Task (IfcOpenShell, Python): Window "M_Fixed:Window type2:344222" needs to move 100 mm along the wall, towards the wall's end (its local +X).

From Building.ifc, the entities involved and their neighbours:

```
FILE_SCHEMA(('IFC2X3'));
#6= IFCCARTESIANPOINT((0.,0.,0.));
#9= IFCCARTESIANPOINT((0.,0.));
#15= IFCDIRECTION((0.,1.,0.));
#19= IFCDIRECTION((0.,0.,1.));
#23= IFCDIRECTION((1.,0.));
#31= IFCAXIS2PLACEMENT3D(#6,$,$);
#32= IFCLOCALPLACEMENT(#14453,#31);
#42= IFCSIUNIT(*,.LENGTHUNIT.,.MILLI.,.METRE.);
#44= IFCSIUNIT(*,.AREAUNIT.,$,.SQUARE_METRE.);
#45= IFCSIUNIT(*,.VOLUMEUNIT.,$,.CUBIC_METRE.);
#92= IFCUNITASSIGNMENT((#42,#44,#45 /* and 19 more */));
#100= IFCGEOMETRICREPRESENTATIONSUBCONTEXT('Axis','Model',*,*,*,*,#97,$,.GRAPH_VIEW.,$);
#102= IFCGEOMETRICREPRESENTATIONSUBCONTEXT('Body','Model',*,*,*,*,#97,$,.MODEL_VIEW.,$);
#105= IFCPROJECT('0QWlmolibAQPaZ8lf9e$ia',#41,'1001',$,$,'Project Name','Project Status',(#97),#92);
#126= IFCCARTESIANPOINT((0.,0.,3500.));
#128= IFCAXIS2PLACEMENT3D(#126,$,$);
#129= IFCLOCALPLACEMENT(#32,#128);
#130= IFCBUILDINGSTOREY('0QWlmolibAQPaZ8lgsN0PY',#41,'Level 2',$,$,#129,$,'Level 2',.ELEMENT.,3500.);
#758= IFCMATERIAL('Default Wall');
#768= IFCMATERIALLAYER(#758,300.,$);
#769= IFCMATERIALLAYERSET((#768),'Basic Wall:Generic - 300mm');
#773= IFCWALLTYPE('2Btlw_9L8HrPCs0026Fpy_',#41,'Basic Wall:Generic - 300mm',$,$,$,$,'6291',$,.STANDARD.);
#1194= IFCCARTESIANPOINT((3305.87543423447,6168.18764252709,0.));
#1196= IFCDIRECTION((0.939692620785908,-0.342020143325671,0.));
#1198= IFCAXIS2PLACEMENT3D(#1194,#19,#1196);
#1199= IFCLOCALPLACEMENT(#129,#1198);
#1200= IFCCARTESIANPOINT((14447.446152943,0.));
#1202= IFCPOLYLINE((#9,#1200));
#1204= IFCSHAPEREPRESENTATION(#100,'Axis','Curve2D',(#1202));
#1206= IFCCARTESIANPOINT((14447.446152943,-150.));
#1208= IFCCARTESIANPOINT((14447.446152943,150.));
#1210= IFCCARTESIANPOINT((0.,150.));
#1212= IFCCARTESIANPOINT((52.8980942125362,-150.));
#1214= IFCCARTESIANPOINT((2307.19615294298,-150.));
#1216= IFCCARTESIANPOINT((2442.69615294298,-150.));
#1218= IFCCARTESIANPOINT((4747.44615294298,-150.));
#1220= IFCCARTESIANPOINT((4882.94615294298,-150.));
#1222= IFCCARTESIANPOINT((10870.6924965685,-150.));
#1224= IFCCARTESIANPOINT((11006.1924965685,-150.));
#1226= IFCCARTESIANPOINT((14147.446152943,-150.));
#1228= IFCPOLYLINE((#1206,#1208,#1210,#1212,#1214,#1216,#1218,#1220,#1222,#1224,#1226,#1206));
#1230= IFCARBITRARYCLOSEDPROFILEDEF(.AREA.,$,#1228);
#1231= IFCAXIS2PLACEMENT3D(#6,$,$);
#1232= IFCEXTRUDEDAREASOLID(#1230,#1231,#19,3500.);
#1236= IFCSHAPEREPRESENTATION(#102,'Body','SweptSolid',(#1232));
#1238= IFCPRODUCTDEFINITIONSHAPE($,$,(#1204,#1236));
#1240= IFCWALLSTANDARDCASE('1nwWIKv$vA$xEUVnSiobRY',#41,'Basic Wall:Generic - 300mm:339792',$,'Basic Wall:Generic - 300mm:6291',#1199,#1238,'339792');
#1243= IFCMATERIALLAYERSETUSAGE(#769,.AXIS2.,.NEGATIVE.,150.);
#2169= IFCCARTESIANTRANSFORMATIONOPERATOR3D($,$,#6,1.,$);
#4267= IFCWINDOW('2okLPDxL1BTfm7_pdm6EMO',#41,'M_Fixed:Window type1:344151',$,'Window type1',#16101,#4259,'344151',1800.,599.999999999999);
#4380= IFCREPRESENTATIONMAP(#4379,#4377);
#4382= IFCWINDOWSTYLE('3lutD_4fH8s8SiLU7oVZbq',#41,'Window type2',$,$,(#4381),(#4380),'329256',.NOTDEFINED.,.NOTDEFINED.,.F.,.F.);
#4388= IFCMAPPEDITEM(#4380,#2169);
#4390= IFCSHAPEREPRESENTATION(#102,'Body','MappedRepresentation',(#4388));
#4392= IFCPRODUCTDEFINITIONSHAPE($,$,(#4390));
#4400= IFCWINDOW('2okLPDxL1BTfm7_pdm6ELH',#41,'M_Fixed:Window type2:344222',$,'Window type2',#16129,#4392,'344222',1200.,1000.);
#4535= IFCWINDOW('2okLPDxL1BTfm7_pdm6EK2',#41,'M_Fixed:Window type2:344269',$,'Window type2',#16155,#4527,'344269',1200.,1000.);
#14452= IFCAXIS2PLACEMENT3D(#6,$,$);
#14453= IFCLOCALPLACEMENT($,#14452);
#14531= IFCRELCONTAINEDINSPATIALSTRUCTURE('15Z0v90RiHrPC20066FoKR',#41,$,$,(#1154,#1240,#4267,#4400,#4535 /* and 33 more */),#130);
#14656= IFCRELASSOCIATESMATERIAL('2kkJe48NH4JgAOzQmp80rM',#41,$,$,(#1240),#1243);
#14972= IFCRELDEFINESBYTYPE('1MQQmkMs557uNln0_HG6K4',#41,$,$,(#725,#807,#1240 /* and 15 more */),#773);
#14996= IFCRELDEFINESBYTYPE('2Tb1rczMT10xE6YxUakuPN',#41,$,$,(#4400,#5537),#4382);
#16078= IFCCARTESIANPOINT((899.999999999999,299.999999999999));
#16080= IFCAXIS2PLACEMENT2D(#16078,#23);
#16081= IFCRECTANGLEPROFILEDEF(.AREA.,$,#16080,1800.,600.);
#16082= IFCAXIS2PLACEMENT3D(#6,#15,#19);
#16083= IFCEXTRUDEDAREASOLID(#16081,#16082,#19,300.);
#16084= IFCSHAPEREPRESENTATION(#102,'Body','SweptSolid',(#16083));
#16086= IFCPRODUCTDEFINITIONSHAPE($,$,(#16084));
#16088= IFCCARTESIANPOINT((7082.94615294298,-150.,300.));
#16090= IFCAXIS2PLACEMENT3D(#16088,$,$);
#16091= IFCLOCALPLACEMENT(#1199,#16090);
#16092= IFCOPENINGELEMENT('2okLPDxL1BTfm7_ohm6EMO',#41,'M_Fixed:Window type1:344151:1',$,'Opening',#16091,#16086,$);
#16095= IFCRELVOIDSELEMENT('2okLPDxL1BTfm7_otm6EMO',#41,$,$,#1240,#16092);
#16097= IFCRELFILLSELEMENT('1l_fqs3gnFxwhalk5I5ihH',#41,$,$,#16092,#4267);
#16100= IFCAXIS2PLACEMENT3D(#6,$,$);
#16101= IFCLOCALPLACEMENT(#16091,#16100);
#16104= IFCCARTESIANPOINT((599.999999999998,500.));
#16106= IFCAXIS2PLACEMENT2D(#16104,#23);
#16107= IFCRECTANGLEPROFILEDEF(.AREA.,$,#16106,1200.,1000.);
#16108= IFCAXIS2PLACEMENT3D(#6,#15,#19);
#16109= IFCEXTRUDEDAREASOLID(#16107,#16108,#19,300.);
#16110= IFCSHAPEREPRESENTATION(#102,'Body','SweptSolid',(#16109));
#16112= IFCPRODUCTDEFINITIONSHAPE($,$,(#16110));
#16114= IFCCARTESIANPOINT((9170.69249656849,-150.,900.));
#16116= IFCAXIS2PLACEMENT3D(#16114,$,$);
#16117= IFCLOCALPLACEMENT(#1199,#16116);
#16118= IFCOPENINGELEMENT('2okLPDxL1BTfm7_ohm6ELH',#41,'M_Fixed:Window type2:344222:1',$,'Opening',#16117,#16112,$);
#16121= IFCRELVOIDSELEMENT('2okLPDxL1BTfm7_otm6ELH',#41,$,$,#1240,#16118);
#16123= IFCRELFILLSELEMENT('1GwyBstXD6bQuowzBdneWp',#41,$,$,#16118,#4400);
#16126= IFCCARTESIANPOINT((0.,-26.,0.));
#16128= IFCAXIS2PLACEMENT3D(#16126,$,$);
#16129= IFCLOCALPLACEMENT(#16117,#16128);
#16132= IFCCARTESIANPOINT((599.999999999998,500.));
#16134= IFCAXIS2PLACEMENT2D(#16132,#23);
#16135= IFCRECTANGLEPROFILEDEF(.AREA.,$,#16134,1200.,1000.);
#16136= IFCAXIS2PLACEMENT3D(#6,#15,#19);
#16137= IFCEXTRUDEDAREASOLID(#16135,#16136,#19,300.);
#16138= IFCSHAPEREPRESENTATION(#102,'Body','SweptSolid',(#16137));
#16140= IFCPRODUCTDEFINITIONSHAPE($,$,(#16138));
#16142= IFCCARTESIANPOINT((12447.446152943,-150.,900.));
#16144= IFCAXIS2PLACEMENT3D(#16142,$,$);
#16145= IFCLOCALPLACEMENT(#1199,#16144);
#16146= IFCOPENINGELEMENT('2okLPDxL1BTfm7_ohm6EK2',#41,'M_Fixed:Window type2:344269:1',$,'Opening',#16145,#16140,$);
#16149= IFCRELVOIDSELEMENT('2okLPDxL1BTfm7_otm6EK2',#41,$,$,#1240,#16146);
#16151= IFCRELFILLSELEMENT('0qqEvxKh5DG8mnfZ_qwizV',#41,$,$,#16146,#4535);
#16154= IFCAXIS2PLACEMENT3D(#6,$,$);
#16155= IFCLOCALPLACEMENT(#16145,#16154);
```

```python
import ifcopenshell
import ifcopenshell.api.geometry
import ifcopenshell.util.placement
import ifcopenshell.util.unit

model = ifcopenshell.open("Building.ifc")
unit_scale = ifcopenshell.util.unit.calculate_unit_scale(model)

window = model.by_id(4400)
opening = window.FillsVoids[0].RelatingOpeningElement
wall = opening.VoidsElements[0].RelatingBuildingElement

wall_matrix = ifcopenshell.util.placement.get_local_placement(wall.ObjectPlacement)
shift = wall_matrix[:3, 0] * 0.1 / unit_scale
before = ifcopenshell.util.placement.get_local_placement(window.ObjectPlacement)[:3, 3].copy()

# The window is placed relative to its opening, so it follows when the opening moves.
matrix = ifcopenshell.util.placement.get_local_placement(opening.ObjectPlacement)
matrix[:3, 3] += shift
ifcopenshell.api.geometry.edit_object_placement(
    model, product=opening, matrix=matrix, is_si=False, should_transform_children=True
)

after = ifcopenshell.util.placement.get_local_placement(window.ObjectPlacement)[:3, 3]
print("window moved by", (after - before).round(3) + 0.0)

model.write("Building_edited.ifc")
```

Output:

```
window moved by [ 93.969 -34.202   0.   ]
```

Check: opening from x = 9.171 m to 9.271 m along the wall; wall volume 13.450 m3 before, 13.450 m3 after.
